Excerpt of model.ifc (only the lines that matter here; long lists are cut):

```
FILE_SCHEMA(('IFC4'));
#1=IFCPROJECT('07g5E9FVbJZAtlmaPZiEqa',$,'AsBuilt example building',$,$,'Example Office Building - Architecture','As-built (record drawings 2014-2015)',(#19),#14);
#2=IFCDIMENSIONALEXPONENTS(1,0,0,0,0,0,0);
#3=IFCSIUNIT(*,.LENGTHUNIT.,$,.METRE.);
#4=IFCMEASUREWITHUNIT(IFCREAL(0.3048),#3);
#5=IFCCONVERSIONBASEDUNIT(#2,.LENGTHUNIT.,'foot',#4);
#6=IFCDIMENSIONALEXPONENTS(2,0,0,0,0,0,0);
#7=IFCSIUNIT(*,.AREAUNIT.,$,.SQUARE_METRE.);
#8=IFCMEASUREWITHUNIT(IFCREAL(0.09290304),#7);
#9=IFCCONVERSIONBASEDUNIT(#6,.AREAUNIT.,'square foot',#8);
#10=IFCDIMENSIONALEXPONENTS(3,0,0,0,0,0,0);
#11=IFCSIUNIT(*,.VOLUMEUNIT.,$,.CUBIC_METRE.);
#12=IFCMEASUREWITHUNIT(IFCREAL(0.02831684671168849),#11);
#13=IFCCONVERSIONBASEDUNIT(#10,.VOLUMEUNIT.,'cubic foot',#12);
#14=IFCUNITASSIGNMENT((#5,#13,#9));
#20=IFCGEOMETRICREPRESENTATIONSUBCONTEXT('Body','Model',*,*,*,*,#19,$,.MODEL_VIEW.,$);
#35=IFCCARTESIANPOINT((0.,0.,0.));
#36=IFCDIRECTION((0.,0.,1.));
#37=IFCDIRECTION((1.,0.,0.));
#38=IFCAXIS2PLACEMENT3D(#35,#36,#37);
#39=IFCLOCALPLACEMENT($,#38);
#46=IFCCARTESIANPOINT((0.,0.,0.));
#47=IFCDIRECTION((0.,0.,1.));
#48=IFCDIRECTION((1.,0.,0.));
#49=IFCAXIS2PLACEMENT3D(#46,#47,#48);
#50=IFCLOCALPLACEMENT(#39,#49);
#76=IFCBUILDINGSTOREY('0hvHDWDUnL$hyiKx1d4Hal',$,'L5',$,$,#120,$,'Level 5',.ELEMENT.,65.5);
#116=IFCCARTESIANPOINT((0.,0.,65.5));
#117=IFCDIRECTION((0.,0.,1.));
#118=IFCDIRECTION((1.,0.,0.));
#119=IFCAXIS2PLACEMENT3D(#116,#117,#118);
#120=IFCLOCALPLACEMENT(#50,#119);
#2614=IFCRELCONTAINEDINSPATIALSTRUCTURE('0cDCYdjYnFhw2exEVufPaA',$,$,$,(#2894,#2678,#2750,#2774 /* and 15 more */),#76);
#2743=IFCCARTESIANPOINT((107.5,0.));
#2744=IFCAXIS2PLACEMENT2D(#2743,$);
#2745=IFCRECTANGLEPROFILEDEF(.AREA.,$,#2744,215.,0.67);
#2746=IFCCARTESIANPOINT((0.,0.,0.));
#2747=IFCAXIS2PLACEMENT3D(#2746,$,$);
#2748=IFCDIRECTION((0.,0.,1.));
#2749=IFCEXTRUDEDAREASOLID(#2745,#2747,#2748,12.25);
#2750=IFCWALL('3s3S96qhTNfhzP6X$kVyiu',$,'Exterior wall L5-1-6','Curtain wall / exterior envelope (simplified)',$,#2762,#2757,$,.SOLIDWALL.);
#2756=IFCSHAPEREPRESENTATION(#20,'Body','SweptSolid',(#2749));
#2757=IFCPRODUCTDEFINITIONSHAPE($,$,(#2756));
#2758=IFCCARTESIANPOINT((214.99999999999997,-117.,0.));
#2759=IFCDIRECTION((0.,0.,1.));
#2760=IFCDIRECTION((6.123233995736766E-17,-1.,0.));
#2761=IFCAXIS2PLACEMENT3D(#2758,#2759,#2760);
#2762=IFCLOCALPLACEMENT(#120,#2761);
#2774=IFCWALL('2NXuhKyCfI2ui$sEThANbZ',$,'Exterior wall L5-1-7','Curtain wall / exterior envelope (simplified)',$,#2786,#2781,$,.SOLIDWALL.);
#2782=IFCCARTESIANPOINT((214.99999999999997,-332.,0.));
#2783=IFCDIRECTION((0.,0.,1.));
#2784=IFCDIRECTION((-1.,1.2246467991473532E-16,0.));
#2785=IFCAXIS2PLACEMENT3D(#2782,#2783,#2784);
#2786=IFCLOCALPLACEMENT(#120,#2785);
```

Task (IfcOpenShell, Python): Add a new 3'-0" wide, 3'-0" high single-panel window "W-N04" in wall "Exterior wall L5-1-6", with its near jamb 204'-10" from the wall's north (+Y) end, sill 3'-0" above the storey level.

```python
import numpy as np
import ifcopenshell
import ifcopenshell.api.feature
import ifcopenshell.api.geometry
import ifcopenshell.api.root
import ifcopenshell.api.spatial
import ifcopenshell.geom
import ifcopenshell.util.element
import ifcopenshell.util.placement
import ifcopenshell.util.representation
import ifcopenshell.util.shape
import ifcopenshell.util.unit

model = ifcopenshell.open("model.ifc")
unit_scale = ifcopenshell.util.unit.calculate_unit_scale(model)
settings = ifcopenshell.geom.settings()


def volume(element):
    """Net volume in cubic metres, openings subtracted."""
    shape = ifcopenshell.geom.create_shape(settings, element)
    return ifcopenshell.util.shape.get_volume(shape.geometry)


wall = model.by_guid("3s3S96qhTNfhzP6X$kVyiu")
storey = ifcopenshell.util.element.get_container(wall, ifc_class="IfcBuildingStorey")
context = ifcopenshell.util.representation.get_context(model, "Model", "Body", "MODEL_VIEW")
before = volume(wall)

width, height, from_end, sill = 0.9144, 0.9144, 62.4332, 0.9144  # metres

# The wall runs along its own X axis, and the end named is its -X end.
wall_shape = ifcopenshell.geom.create_shape(settings, wall)
x, y, z = ifcopenshell.util.shape.get_vertices(wall_shape.geometry).T
start = x.min() + from_end
face, thickness = float(y.min()), float(y.max() - y.min())
wall_matrix = ifcopenshell.util.placement.get_local_placement(wall.ObjectPlacement)
level = ifcopenshell.util.placement.get_local_placement(storey.ObjectPlacement)[2, 3]


def in_wall(x, y):
    """Placement at x, y metres in the wall's axes, at sill height."""
    matrix = wall_matrix.copy()
    matrix[:, 3] = wall_matrix @ np.array([x / unit_scale, y / unit_scale, 0.0, 1.0])
    matrix[2, 3] = level + sill / unit_scale
    return matrix


# Opening: a box that overshoots both wall faces by 50 mm.
opening = ifcopenshell.api.root.create_entity(model, ifc_class="IfcOpeningElement", predefined_type="OPENING")
box = ifcopenshell.api.geometry.add_wall_representation(
    model, context=context, length=width, height=height, thickness=thickness + 0.1
)
ifcopenshell.api.geometry.assign_representation(model, product=opening, representation=box)
ifcopenshell.api.geometry.edit_object_placement(model, product=opening, matrix=in_wall(start, face - 0.05), is_si=False)
ifcopenshell.api.feature.add_feature(model, feature=opening, element=wall)

window = ifcopenshell.api.root.create_entity(model, ifc_class="IfcWindow", name="W-N04", predefined_type="WINDOW")
window.OverallWidth, window.OverallHeight = width / unit_scale, height / unit_scale
window.PartitioningType = "SINGLE_PANEL"
body = ifcopenshell.api.geometry.add_window_representation(
    model,
    context=context,
    overall_width=window.OverallWidth,
    overall_height=window.OverallHeight,
    partition_type="SINGLE_PANEL",
)
ifcopenshell.api.geometry.assign_representation(model, product=window, representation=body)
ifcopenshell.api.spatial.assign_container(model, products=[window], relating_structure=storey)
ifcopenshell.api.feature.add_filling(model, opening=opening, element=window)

# Centre the window in the wall's thickness.
ifcopenshell.api.geometry.edit_object_placement(model, product=window, matrix=in_wall(start, face), is_si=False)
window_shape = ifcopenshell.geom.create_shape(settings, window)
depth = ifcopenshell.util.shape.get_vertices(window_shape.geometry)[:, 1]
offset = face + thickness / 2 - (depth.min() + depth.max()) / 2
ifcopenshell.api.geometry.edit_object_placement(model, product=window, matrix=in_wall(start, offset), is_si=False)

after = volume(wall)

print(f"wall volume {before:.3f} -> {after:.3f} m3")

model.write("model_v2.ifc")
```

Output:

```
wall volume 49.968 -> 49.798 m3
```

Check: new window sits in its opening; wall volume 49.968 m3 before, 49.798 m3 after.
